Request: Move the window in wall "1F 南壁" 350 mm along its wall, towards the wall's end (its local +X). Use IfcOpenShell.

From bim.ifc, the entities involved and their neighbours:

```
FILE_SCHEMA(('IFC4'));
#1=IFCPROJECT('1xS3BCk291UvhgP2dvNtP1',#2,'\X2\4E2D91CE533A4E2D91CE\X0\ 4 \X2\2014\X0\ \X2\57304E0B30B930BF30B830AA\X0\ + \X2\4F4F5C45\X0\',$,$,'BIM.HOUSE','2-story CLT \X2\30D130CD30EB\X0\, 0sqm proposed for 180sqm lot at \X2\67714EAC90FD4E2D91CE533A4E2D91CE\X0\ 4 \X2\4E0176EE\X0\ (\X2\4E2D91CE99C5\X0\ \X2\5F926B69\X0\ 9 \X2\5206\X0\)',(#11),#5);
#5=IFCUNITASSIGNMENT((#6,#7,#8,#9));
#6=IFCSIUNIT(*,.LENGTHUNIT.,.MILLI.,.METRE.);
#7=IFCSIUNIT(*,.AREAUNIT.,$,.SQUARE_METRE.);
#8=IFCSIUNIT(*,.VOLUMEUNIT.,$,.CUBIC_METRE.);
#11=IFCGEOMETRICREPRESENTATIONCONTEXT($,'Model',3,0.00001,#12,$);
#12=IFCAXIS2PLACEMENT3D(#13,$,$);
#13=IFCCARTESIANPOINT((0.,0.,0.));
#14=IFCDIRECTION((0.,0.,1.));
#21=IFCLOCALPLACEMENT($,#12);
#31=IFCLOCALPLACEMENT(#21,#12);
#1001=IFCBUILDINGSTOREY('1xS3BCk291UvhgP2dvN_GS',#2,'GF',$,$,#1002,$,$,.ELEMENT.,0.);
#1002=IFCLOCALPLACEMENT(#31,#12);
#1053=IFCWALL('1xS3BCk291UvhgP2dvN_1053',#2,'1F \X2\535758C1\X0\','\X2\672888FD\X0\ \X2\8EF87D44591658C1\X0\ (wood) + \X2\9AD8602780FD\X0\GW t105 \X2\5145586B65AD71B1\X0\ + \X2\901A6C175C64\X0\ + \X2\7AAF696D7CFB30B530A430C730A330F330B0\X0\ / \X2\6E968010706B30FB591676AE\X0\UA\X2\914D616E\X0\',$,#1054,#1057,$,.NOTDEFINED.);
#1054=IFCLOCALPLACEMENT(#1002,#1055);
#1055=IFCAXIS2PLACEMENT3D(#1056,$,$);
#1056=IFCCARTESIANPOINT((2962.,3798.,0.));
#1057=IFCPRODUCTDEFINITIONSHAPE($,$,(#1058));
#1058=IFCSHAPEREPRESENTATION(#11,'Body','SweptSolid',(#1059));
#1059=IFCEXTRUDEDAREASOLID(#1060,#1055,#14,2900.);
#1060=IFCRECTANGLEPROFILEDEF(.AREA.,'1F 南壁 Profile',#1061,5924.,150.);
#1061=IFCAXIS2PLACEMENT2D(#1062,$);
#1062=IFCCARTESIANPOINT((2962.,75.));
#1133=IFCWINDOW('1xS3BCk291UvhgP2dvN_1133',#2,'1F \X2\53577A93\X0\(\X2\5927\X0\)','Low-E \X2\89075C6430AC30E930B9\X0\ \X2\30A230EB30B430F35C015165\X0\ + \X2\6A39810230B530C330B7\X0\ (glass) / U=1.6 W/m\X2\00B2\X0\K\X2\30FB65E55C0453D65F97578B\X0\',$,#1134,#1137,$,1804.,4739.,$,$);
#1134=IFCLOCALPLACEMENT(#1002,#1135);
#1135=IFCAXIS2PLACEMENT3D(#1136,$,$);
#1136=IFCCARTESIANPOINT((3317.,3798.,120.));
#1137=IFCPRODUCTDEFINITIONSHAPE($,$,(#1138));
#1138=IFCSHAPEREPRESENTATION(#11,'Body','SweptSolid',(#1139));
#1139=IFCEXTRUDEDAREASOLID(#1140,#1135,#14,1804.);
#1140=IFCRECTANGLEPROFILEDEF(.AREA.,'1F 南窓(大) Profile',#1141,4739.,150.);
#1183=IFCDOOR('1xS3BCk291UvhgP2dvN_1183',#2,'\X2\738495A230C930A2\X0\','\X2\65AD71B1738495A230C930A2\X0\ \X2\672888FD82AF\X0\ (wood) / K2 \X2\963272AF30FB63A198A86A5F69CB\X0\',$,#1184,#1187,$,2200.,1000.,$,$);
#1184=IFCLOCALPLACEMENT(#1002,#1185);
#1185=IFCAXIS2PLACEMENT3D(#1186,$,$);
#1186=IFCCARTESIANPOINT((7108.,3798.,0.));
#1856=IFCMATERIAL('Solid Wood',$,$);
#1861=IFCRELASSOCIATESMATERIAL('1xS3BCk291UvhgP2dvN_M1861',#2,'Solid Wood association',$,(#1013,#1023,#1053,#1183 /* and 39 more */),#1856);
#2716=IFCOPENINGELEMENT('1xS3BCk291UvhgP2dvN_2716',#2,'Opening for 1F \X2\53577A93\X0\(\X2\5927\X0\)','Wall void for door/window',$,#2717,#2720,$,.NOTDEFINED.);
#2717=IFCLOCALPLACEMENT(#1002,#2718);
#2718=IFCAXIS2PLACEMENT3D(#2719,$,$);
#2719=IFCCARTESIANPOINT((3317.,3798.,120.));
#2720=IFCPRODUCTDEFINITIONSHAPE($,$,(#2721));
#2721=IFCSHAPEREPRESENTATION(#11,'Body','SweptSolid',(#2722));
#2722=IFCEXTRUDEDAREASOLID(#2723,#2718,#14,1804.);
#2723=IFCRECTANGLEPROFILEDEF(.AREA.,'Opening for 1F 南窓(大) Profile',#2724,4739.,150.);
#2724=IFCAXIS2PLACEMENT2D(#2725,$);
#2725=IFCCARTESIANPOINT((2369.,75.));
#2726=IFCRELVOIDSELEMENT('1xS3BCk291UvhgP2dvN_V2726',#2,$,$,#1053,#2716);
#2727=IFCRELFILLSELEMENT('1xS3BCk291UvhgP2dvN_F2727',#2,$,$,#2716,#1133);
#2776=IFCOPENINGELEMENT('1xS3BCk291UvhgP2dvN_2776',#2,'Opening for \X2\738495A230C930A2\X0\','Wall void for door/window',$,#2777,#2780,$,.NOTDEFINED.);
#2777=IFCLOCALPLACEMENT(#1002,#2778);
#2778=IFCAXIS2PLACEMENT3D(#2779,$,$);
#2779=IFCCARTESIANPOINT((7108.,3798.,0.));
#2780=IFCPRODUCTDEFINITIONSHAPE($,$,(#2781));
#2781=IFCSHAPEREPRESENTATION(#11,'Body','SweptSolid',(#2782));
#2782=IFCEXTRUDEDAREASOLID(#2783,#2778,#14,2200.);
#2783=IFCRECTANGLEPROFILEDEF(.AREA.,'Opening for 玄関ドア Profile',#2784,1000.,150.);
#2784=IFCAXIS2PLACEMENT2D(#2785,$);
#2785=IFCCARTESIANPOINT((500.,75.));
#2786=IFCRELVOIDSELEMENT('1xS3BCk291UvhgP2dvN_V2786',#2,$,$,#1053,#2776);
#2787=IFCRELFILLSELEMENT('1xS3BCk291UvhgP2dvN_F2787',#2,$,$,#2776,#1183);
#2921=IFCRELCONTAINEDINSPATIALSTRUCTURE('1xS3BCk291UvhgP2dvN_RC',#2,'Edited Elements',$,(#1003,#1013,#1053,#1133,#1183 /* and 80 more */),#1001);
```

```python
import ifcopenshell
import ifcopenshell.api.geometry
import ifcopenshell.util.placement
import ifcopenshell.util.unit

model = ifcopenshell.open("bim.ifc")
unit_scale = ifcopenshell.util.unit.calculate_unit_scale(model)

window = model.by_guid("1xS3BCk291UvhgP2dvN_1133")
opening = window.FillsVoids[0].RelatingOpeningElement
wall = opening.VoidsElements[0].RelatingBuildingElement

wall_matrix = ifcopenshell.util.placement.get_local_placement(wall.ObjectPlacement)
shift = wall_matrix[:3, 0] * 0.35 / unit_scale
before = ifcopenshell.util.placement.get_local_placement(window.ObjectPlacement)[:3, 3].copy()

# The window is not placed relative to its opening, so move both.
for product in (opening, window):
    matrix = ifcopenshell.util.placement.get_local_placement(product.ObjectPlacement)
    matrix[:3, 3] += shift
    ifcopenshell.api.geometry.edit_object_placement(model, product=product, matrix=matrix, is_si=False)

after = ifcopenshell.util.placement.get_local_placement(window.ObjectPlacement)[:3, 3]
print("window moved by", (after - before).round(3) + 0.0)

model.write("bim-out.ifc")
```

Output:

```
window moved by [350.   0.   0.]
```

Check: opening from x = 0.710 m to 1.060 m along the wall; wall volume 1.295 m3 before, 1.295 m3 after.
